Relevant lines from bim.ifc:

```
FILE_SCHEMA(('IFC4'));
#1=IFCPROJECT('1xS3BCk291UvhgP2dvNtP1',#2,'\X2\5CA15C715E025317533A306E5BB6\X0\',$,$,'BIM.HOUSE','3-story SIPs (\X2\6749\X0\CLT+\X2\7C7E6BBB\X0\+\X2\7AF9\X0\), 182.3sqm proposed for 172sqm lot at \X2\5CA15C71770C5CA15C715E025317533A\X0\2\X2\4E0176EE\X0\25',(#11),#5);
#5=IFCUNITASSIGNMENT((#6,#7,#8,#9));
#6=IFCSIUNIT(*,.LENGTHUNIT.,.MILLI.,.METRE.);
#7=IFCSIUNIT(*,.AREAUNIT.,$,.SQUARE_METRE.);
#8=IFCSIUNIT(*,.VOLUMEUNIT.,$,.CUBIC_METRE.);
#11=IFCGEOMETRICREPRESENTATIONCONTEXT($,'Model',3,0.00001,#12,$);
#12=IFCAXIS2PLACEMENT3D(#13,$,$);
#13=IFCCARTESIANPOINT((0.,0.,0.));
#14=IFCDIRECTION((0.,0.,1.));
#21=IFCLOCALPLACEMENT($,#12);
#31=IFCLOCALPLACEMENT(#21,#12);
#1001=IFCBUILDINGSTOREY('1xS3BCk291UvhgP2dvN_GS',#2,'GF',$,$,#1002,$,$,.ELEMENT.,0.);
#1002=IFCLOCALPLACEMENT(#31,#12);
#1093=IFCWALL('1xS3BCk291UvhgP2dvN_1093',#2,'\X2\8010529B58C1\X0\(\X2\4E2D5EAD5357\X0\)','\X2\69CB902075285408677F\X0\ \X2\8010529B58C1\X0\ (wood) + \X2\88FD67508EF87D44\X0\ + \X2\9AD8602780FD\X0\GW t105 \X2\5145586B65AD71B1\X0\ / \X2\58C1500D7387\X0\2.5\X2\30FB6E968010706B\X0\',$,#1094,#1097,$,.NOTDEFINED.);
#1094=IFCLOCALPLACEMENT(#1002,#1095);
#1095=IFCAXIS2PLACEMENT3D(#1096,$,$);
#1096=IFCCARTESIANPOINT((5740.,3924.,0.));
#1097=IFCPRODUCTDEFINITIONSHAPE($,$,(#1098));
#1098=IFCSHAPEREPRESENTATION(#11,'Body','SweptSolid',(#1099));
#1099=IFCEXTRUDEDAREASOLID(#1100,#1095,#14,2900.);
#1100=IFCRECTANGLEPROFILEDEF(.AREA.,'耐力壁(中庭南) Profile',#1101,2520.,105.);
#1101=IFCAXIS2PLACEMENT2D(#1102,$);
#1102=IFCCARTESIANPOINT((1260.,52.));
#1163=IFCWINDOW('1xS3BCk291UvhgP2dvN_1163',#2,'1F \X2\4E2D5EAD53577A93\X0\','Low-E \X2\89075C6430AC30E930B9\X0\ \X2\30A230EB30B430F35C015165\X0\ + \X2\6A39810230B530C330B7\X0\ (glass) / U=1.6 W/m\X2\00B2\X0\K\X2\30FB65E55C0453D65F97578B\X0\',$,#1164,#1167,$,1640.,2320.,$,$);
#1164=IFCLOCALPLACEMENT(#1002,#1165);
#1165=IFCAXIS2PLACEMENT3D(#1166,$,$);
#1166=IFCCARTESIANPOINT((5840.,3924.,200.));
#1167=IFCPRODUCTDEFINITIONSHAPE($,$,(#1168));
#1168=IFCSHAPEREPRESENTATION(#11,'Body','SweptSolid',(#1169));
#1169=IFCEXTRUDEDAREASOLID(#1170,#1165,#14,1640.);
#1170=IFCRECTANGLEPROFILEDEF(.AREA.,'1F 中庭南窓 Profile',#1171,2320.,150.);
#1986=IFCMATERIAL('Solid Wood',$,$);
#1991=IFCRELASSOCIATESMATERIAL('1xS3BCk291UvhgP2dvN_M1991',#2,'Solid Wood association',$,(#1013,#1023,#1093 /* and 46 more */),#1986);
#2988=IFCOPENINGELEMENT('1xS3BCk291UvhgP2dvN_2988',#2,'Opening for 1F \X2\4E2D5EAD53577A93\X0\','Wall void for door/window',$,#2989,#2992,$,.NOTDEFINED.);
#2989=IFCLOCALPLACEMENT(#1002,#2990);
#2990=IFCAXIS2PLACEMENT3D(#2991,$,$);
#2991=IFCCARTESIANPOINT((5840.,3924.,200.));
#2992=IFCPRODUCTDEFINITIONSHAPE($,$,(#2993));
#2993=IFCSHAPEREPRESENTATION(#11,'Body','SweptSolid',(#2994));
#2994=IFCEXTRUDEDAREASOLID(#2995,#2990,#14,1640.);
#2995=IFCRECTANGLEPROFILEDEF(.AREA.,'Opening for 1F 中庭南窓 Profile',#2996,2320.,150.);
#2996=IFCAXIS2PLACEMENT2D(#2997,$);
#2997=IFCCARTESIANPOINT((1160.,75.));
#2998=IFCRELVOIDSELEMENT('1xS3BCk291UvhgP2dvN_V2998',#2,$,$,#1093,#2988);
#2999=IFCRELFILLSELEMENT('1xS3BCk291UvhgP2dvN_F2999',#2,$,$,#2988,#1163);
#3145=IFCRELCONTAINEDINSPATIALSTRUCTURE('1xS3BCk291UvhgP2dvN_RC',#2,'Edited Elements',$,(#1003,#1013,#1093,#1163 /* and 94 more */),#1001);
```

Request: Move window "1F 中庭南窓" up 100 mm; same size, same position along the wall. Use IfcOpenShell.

```python
import numpy as np
import ifcopenshell
import ifcopenshell.api.geometry
import ifcopenshell.util.placement
import ifcopenshell.util.unit

model = ifcopenshell.open("bim.ifc")
unit_scale = ifcopenshell.util.unit.calculate_unit_scale(model)

window = model.by_id(1163)
opening = window.FillsVoids[0].RelatingOpeningElement
dz = 0.1 / unit_scale

shift = np.array([0.0, 0.0, dz])
# The window is not placed relative to its opening, so move both.
for product in (opening, window):
    matrix = ifcopenshell.util.placement.get_local_placement(product.ObjectPlacement)
    matrix[:3, 3] += shift
    ifcopenshell.api.geometry.edit_object_placement(model, product=product, matrix=matrix, is_si=False)

print(f"moved by {dz * unit_scale:+.3f} m")

model.write("bim-out.ifc")
```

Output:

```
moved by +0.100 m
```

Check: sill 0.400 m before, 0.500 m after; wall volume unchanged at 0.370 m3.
